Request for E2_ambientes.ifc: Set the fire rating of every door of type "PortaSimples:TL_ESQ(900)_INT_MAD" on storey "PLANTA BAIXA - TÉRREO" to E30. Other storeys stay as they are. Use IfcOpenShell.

First a look at what the model holds.

```python
import ifcopenshell
import ifcopenshell.util.element

model = ifcopenshell.open("E2_ambientes.ifc")
print(model.schema)
storey = next(s for s in model.by_type("IfcBuildingStorey") if s.Name == "PLANTA BAIXA - TÉRREO")
doors = [e for e in ifcopenshell.util.element.get_decomposition(storey) if e.is_a("IfcDoor")]
seen = {}
for e in doors:
    element_type = ifcopenshell.util.element.get_type(e)
    key = (element_type.Name if element_type != e and element_type else None, ifcopenshell.util.element.get_pset(e, "Pset_DoorCommon", "FireRating"))
    seen[key] = seen.get(key, 0) + 1
for (name, value), count in sorted(seen.items(), key=str):
    print(count, "x", name, "|", value)
```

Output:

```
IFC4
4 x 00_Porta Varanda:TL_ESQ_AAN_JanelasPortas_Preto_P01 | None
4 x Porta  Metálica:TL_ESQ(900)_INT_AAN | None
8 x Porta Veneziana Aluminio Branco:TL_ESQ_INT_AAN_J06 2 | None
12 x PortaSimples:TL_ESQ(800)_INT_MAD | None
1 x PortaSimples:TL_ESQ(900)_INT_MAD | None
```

```python
import ifcopenshell
import ifcopenshell.api.pset
import ifcopenshell.util.element

model = ifcopenshell.open("E2_ambientes.ifc")

storey = next(s for s in model.by_type("IfcBuildingStorey") if s.Name == "PLANTA BAIXA - TÉRREO")
doors = [e for e in ifcopenshell.util.element.get_decomposition(storey) if e.is_a("IfcDoor")]

count = 0
for e in doors:
    element_type = ifcopenshell.util.element.get_type(e)
    if element_type in (None, e) or element_type.Name != "PortaSimples:TL_ESQ(900)_INT_MAD":
        continue
    # add_pset returns the element's existing set when there is one.
    pset = ifcopenshell.api.pset.add_pset(model, product=e, name="Pset_DoorCommon")
    ifcopenshell.api.pset.edit_pset(model, pset=pset, properties={"FireRating": "E30"})
    count += 1

print(count, "doors updated")

model.write("E2_ambientes_updated.ifc")
```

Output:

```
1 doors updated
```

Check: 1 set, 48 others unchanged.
